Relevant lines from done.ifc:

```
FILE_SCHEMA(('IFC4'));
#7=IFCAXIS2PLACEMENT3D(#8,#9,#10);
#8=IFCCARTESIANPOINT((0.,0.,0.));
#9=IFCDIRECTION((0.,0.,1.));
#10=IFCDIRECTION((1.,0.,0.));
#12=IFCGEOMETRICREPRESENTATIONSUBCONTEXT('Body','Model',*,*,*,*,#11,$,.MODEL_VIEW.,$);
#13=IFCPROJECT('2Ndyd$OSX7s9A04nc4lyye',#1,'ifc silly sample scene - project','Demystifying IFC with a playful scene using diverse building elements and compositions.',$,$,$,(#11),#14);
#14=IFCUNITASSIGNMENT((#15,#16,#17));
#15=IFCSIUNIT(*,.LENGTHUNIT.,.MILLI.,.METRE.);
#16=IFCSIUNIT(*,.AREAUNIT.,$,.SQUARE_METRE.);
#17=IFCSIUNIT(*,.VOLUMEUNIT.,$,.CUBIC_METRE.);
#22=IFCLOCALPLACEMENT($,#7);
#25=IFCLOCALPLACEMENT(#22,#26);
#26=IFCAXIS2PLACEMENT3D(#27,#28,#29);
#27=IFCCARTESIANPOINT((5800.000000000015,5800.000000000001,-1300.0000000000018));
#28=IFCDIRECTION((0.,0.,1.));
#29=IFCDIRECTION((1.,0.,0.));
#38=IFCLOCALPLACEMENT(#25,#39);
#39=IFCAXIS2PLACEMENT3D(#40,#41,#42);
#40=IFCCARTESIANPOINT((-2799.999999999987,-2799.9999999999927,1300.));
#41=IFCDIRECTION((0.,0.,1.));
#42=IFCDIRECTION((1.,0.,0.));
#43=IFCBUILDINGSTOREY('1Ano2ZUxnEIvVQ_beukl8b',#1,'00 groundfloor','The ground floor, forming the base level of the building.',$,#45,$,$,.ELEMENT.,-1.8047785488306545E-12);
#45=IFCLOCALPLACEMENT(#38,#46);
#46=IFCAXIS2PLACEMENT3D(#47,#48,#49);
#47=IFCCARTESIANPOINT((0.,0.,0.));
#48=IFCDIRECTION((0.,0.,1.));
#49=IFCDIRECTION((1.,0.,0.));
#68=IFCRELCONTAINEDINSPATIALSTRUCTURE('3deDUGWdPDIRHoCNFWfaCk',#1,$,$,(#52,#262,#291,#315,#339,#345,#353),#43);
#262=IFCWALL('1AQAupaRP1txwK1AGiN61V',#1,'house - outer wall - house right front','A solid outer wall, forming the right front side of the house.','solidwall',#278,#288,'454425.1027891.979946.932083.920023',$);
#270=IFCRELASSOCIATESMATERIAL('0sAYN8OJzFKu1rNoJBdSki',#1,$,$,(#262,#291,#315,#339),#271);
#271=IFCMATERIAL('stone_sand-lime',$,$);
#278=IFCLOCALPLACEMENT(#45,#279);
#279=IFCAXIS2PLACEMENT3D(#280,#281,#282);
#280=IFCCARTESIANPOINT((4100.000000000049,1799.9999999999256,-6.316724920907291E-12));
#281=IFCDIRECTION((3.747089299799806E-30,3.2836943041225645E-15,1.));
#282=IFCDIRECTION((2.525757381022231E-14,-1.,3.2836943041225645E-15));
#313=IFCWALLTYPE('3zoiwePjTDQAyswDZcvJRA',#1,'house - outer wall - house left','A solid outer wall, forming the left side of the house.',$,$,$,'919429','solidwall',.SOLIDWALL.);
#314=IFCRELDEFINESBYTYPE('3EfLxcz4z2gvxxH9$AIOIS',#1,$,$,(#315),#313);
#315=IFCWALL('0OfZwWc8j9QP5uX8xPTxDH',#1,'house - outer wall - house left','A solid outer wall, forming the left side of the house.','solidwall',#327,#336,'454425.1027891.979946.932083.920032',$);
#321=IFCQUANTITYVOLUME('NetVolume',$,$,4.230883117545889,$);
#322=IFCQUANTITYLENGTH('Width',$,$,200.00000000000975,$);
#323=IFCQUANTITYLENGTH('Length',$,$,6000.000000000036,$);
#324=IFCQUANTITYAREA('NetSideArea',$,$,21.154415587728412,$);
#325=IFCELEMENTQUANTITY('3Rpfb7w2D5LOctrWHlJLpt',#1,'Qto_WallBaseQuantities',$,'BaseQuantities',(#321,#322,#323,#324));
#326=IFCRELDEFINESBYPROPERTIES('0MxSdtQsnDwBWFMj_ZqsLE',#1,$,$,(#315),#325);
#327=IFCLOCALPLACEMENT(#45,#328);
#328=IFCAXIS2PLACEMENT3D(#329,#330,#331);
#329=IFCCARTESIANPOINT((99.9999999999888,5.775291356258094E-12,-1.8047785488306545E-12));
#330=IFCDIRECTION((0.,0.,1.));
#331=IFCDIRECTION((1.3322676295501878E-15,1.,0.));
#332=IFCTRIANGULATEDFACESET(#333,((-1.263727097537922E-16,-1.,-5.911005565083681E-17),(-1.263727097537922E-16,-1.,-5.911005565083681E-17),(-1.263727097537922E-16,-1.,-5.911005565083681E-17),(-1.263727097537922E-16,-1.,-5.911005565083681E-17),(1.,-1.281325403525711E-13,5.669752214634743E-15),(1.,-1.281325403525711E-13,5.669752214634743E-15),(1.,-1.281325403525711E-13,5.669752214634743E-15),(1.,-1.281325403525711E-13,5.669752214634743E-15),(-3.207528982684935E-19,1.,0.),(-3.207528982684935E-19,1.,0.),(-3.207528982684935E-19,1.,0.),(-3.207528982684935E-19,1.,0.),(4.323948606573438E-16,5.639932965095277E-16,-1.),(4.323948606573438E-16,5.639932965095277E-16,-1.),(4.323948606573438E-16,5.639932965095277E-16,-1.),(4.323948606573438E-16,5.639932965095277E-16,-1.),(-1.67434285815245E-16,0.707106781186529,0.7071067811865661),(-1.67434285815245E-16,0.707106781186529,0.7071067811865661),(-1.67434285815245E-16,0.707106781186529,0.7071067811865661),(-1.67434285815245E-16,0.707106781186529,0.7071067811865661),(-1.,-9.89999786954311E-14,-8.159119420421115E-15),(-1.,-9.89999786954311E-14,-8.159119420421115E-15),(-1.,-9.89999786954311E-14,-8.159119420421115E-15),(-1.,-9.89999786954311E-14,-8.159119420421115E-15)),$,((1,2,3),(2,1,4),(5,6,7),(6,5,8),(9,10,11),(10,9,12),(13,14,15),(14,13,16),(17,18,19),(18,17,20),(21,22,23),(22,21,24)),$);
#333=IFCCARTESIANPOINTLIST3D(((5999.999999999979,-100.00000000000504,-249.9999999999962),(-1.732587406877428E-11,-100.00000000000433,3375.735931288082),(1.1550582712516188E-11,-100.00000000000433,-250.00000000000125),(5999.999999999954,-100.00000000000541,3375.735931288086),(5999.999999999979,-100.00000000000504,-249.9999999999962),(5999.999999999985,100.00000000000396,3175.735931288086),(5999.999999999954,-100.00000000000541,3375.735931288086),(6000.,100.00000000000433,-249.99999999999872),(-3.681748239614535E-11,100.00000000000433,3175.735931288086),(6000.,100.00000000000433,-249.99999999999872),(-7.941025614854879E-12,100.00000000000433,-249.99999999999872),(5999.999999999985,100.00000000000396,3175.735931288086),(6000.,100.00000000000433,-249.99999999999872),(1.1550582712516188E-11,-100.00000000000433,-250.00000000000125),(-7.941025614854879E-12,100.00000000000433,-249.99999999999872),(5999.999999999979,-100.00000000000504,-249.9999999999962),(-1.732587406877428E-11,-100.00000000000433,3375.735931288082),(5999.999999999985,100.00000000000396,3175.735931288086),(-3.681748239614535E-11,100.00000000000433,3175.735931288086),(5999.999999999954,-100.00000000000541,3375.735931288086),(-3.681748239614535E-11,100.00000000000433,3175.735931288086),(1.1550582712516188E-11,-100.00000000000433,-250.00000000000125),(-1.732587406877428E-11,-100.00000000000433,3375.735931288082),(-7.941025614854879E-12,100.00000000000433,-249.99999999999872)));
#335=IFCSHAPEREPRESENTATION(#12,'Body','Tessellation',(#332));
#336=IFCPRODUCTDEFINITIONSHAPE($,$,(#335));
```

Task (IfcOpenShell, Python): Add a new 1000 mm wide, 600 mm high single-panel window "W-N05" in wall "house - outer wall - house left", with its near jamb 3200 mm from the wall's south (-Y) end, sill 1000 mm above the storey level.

```python
import numpy as np
import ifcopenshell
import ifcopenshell.api.feature
import ifcopenshell.api.geometry
import ifcopenshell.api.pset
import ifcopenshell.api.root
import ifcopenshell.api.spatial
import ifcopenshell.geom
import ifcopenshell.util.element
import ifcopenshell.util.placement
import ifcopenshell.util.representation
import ifcopenshell.util.shape
import ifcopenshell.util.unit

model = ifcopenshell.open("done.ifc")
unit_scale = ifcopenshell.util.unit.calculate_unit_scale(model)
area_scale = ifcopenshell.util.unit.calculate_unit_scale(model, "AREAUNIT")
volume_scale = ifcopenshell.util.unit.calculate_unit_scale(model, "VOLUMEUNIT")
settings = ifcopenshell.geom.settings()


def volume(element):
    """Net volume in cubic metres, openings subtracted."""
    shape = ifcopenshell.geom.create_shape(settings, element)
    return ifcopenshell.util.shape.get_volume(shape.geometry)


wall = model.by_id(315)
storey = ifcopenshell.util.element.get_container(wall, ifc_class="IfcBuildingStorey")
context = ifcopenshell.util.representation.get_context(model, "Model", "Body", "MODEL_VIEW")
before = volume(wall)

width, height, from_end, sill = 1, 0.6, 3.2, 1  # metres

# The wall runs along its own X axis, and the end named is its -X end.
wall_shape = ifcopenshell.geom.create_shape(settings, wall)
x, y, z = ifcopenshell.util.shape.get_vertices(wall_shape.geometry).T
start = x.min() + from_end
face, thickness = float(y.min()), float(y.max() - y.min())
wall_matrix = ifcopenshell.util.placement.get_local_placement(wall.ObjectPlacement)
level = ifcopenshell.util.placement.get_local_placement(storey.ObjectPlacement)[2, 3]


def in_wall(x, y):
    """Placement at x, y metres in the wall's axes, at sill height."""
    matrix = wall_matrix.copy()
    matrix[:, 3] = wall_matrix @ np.array([x / unit_scale, y / unit_scale, 0.0, 1.0])
    matrix[2, 3] = level + sill / unit_scale
    return matrix


# Opening: a box that overshoots both wall faces by 50 mm.
opening = ifcopenshell.api.root.create_entity(model, ifc_class="IfcOpeningElement", predefined_type="OPENING")
box = ifcopenshell.api.geometry.add_wall_representation(
    model, context=context, length=width, height=height, thickness=thickness + 0.1
)
ifcopenshell.api.geometry.assign_representation(model, product=opening, representation=box)
ifcopenshell.api.geometry.edit_object_placement(model, product=opening, matrix=in_wall(start, face - 0.05), is_si=False)
ifcopenshell.api.feature.add_feature(model, feature=opening, element=wall)

window = ifcopenshell.api.root.create_entity(model, ifc_class="IfcWindow", name="W-N05", predefined_type="WINDOW")
window.OverallWidth, window.OverallHeight = width / unit_scale, height / unit_scale
window.PartitioningType = "SINGLE_PANEL"
body = ifcopenshell.api.geometry.add_window_representation(
    model,
    context=context,
    overall_width=window.OverallWidth,
    overall_height=window.OverallHeight,
    partition_type="SINGLE_PANEL",
)
ifcopenshell.api.geometry.assign_representation(model, product=window, representation=body)
ifcopenshell.api.spatial.assign_container(model, products=[window], relating_structure=storey)
ifcopenshell.api.feature.add_filling(model, opening=opening, element=window)

# Centre the window in the wall's thickness.
ifcopenshell.api.geometry.edit_object_placement(model, product=window, matrix=in_wall(start, face), is_si=False)
window_shape = ifcopenshell.geom.create_shape(settings, window)
depth = ifcopenshell.util.shape.get_vertices(window_shape.geometry)[:, 1]
offset = face + thickness / 2 - (depth.min() + depth.max()) / 2
ifcopenshell.api.geometry.edit_object_placement(model, product=window, matrix=in_wall(start, offset), is_si=False)

after = volume(wall)

# Update the wall's stored quantities.
qto = model.by_id(ifcopenshell.util.element.get_pset(wall, "Qto_WallBaseQuantities", should_inherit=False)["id"])
ifcopenshell.api.pset.edit_qto(model, qto=qto, properties={
    "NetVolume": after / volume_scale,
    "NetSideArea": after / thickness / area_scale,
})

print(f"wall volume {before:.3f} -> {after:.3f} m3")

model.write("done_rev.ifc")
```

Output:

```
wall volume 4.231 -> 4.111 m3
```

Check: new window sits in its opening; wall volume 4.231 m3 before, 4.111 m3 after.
